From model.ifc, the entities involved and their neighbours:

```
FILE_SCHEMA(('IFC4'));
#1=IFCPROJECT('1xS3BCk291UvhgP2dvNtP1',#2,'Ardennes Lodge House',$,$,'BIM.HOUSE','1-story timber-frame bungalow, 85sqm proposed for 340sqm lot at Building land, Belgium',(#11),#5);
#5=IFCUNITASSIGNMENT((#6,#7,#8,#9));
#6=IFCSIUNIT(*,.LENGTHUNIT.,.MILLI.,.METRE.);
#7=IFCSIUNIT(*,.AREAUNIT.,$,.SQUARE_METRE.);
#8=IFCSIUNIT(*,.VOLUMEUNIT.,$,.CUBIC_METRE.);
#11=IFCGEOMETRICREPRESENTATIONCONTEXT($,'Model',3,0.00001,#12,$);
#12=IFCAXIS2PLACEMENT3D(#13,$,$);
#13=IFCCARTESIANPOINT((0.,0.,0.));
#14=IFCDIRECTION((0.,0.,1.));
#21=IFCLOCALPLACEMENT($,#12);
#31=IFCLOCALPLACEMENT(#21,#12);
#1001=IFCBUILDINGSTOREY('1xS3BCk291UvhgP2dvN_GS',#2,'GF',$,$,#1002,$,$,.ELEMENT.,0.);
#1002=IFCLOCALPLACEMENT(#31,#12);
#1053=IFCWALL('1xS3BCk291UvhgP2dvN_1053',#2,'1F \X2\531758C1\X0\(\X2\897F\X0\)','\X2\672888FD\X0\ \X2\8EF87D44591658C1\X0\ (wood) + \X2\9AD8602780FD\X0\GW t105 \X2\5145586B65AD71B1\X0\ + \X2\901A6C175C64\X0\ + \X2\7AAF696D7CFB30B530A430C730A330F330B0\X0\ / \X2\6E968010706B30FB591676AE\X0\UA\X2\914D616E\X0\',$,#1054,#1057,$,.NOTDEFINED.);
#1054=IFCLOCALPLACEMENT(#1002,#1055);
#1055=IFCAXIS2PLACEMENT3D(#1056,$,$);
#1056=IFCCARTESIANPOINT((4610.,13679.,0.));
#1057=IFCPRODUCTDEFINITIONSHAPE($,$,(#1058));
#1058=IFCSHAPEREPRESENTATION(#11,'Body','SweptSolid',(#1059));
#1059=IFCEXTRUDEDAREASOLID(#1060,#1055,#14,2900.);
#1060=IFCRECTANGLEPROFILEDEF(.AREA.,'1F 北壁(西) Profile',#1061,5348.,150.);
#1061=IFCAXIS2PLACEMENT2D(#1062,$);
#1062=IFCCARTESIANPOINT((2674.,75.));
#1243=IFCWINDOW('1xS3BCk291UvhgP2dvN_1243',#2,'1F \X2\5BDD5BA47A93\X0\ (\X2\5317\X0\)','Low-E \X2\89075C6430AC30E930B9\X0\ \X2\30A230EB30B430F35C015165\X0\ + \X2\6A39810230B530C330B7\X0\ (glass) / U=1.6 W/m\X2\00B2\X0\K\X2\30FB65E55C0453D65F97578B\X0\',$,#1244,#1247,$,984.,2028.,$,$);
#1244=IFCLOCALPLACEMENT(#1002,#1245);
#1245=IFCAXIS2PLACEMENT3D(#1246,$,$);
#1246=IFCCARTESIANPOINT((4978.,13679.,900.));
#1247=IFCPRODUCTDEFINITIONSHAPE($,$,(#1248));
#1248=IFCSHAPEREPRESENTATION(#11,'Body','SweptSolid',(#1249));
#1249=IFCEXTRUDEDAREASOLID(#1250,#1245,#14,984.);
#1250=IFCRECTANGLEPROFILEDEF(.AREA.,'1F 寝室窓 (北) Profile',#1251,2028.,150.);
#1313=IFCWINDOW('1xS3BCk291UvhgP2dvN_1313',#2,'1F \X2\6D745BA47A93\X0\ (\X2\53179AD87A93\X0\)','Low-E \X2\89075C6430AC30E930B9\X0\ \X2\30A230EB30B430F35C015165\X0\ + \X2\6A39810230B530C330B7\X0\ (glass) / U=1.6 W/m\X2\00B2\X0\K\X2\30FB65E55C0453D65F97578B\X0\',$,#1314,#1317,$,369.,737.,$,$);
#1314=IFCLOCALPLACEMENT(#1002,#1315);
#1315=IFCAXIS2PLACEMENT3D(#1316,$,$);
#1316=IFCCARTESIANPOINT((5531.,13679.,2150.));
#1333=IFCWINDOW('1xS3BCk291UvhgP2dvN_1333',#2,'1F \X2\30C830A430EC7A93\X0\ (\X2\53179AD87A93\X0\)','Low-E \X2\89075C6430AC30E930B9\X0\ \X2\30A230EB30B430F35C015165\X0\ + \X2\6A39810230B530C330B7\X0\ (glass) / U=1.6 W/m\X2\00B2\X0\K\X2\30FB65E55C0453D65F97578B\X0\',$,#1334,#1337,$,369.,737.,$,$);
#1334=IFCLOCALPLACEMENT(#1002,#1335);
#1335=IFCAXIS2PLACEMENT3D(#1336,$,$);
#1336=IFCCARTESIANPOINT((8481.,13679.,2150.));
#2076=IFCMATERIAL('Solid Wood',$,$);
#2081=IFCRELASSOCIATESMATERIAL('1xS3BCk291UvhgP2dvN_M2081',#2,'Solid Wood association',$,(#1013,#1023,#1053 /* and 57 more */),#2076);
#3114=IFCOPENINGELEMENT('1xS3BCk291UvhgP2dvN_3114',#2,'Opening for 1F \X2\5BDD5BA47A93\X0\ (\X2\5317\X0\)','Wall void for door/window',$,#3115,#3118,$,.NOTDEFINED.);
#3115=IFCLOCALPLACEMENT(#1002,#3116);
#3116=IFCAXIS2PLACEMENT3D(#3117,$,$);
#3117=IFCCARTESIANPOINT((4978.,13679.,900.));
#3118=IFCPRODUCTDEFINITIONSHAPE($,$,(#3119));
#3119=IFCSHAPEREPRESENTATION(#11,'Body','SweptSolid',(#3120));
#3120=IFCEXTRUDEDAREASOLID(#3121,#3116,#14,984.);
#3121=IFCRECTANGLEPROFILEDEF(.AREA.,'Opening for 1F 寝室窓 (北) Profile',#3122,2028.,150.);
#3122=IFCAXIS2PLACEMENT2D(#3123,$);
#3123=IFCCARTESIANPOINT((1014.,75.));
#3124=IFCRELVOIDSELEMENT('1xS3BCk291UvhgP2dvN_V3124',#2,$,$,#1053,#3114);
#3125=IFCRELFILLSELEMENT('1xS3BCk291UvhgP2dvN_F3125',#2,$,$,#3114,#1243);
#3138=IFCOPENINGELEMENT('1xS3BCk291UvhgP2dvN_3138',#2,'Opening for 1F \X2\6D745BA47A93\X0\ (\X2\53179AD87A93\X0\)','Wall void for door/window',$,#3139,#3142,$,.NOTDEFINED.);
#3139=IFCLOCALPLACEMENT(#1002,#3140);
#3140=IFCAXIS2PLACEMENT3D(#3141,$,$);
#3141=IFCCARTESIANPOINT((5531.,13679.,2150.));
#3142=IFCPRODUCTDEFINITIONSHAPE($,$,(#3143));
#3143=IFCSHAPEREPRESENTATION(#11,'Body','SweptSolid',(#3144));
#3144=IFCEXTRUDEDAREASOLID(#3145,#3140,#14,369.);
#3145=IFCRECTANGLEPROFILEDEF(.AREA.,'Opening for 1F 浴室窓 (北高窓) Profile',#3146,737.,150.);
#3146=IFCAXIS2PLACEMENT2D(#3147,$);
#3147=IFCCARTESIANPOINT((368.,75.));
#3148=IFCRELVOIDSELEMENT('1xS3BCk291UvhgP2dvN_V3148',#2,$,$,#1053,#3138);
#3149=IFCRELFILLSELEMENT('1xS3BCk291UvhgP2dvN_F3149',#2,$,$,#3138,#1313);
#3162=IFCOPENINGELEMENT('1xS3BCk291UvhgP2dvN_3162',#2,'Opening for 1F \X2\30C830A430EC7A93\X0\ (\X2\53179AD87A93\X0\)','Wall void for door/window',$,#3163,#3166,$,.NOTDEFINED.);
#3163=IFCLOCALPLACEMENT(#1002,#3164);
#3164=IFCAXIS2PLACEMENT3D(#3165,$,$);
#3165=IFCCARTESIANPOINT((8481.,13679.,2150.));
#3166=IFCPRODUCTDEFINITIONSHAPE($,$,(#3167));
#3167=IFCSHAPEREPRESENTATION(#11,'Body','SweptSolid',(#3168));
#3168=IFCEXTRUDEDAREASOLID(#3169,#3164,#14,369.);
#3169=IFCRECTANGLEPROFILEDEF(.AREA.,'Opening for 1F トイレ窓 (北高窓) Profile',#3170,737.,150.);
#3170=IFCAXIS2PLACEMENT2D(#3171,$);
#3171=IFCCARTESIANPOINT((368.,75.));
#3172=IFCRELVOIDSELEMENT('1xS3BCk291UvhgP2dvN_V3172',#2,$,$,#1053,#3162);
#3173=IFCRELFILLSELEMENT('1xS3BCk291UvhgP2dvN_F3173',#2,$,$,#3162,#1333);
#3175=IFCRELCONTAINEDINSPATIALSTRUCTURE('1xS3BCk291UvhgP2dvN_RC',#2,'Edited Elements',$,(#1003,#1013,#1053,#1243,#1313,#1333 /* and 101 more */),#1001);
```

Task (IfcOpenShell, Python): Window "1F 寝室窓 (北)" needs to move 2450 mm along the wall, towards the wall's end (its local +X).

```python
import ifcopenshell
import ifcopenshell.api.geometry
import ifcopenshell.util.placement
import ifcopenshell.util.unit

model = ifcopenshell.open("model.ifc")
unit_scale = ifcopenshell.util.unit.calculate_unit_scale(model)

window = model.by_id(1243)
opening = window.FillsVoids[0].RelatingOpeningElement
wall = opening.VoidsElements[0].RelatingBuildingElement

wall_matrix = ifcopenshell.util.placement.get_local_placement(wall.ObjectPlacement)
shift = wall_matrix[:3, 0] * 2.45 / unit_scale
before = ifcopenshell.util.placement.get_local_placement(window.ObjectPlacement)[:3, 3].copy()

# The window is not placed relative to its opening, so move both.
for product in (opening, window):
    matrix = ifcopenshell.util.placement.get_local_placement(product.ObjectPlacement)
    matrix[:3, 3] += shift
    ifcopenshell.api.geometry.edit_object_placement(model, product=product, matrix=matrix, is_si=False)

after = ifcopenshell.util.placement.get_local_placement(window.ObjectPlacement)[:3, 3]
print("window moved by", (after - before).round(3) + 0.0)

model.write("model_rev.ifc")
```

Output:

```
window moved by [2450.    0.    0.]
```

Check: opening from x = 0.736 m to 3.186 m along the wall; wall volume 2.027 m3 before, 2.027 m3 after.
